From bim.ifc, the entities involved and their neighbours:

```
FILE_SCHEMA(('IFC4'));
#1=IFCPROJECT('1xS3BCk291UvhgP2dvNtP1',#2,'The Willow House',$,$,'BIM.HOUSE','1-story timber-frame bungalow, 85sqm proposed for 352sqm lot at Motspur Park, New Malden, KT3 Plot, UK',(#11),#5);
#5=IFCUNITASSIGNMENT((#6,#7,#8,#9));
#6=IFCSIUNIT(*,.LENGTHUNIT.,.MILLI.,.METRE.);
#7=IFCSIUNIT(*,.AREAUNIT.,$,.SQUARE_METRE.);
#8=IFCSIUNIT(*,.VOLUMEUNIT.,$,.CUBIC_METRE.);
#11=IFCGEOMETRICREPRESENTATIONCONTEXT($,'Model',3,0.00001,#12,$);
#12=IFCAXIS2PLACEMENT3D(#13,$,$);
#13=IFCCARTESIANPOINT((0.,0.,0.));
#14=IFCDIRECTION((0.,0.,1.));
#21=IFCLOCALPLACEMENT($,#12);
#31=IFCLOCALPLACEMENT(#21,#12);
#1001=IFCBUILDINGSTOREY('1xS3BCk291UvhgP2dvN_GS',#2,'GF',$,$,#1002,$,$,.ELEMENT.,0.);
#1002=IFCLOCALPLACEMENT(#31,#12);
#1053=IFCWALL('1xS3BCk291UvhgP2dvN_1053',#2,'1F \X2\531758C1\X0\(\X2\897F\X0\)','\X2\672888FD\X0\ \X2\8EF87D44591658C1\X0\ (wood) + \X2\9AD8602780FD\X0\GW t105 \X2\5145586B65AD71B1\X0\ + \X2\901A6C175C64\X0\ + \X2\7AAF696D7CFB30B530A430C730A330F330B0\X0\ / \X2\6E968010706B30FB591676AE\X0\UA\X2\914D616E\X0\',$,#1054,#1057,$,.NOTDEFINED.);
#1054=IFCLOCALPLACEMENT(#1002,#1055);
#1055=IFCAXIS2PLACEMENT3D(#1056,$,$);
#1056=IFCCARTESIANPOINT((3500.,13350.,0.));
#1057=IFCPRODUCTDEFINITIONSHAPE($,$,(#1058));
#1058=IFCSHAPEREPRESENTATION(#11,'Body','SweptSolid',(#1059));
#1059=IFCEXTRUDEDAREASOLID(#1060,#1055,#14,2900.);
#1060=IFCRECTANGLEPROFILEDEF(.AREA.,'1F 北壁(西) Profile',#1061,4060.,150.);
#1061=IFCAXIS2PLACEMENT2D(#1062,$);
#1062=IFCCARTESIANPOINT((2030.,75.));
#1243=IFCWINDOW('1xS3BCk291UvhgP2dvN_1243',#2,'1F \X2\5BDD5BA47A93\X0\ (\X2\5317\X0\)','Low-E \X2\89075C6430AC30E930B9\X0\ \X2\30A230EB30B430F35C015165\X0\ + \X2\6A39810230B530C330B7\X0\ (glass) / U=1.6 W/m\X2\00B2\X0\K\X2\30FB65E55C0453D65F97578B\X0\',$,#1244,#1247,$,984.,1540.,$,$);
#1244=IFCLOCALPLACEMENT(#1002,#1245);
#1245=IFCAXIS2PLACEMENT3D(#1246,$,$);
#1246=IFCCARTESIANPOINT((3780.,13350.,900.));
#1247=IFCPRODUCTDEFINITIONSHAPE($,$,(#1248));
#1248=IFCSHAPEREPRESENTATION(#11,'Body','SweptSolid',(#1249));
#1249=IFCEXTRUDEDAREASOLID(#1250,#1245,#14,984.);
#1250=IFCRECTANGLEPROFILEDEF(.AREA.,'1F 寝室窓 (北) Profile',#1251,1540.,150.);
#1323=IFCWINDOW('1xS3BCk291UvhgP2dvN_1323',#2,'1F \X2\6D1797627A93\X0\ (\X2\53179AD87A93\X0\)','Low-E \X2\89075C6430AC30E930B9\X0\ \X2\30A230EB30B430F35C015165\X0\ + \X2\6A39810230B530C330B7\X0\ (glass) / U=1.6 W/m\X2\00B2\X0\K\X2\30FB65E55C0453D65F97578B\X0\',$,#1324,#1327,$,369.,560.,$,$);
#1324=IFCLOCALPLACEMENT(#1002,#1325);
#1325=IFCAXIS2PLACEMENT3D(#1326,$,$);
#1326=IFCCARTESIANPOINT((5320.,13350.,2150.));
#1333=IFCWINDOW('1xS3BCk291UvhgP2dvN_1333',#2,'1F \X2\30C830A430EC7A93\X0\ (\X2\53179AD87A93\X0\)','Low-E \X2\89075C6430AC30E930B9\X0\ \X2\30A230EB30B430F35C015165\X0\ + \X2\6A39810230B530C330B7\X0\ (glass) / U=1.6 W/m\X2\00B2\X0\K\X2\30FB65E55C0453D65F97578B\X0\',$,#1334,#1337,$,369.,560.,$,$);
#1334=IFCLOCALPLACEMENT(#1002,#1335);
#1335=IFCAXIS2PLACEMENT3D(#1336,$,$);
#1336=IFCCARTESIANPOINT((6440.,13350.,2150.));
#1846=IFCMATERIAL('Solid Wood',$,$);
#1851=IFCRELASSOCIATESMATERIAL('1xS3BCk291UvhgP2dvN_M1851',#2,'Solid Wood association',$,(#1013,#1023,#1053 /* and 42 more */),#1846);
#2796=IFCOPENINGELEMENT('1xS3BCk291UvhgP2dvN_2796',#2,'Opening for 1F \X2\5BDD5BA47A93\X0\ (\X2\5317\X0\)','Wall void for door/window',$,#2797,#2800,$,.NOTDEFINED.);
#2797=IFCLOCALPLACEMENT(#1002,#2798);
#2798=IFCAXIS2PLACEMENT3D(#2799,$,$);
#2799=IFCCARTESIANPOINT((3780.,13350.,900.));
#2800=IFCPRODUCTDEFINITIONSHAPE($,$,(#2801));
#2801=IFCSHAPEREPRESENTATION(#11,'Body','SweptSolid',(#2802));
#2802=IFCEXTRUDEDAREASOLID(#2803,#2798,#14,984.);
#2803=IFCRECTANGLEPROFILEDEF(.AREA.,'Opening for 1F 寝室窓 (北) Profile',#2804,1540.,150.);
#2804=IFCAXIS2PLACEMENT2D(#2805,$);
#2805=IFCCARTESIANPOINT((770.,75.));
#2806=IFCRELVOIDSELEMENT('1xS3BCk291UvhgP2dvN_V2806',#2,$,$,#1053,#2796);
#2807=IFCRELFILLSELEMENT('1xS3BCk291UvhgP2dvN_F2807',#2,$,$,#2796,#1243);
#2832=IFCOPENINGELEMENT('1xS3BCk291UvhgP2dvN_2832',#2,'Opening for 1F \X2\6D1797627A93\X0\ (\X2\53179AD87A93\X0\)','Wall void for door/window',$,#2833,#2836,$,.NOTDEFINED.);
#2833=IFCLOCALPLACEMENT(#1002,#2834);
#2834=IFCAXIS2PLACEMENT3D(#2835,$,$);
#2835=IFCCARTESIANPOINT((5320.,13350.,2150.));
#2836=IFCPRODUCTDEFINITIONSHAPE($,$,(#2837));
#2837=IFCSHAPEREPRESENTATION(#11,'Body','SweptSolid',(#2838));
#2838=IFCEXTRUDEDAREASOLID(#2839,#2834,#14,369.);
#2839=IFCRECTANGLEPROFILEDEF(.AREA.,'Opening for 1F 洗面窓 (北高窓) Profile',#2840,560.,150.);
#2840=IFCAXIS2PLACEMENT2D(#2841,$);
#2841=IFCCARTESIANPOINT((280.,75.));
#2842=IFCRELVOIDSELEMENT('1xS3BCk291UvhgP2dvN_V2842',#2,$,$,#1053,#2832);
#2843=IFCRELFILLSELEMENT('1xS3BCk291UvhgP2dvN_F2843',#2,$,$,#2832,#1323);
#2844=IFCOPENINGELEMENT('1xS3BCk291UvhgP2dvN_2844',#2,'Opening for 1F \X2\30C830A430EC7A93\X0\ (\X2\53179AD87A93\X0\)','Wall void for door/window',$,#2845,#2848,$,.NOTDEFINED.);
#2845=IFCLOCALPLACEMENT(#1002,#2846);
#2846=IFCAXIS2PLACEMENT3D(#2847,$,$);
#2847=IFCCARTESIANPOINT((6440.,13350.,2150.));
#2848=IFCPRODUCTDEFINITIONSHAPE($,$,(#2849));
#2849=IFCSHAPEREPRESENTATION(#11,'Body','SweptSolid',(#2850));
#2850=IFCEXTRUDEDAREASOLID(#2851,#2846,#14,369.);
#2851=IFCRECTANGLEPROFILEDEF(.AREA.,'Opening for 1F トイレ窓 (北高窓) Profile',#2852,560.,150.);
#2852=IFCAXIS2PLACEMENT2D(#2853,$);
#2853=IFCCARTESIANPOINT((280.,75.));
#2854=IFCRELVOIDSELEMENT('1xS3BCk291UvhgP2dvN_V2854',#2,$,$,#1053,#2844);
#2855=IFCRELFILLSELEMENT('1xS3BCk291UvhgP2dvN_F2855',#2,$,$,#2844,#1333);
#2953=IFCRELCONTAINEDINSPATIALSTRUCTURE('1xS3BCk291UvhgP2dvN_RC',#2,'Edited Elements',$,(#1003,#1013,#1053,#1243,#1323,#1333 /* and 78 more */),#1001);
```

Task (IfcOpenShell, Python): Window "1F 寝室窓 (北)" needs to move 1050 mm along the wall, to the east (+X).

```python
import ifcopenshell
import ifcopenshell.api.geometry
import ifcopenshell.util.placement
import ifcopenshell.util.unit

model = ifcopenshell.open("bim.ifc")
unit_scale = ifcopenshell.util.unit.calculate_unit_scale(model)

window = model.by_guid("1xS3BCk291UvhgP2dvN_1243")
opening = window.FillsVoids[0].RelatingOpeningElement
wall = opening.VoidsElements[0].RelatingBuildingElement

wall_matrix = ifcopenshell.util.placement.get_local_placement(wall.ObjectPlacement)
shift = wall_matrix[:3, 0] * 1.05 / unit_scale
before = ifcopenshell.util.placement.get_local_placement(window.ObjectPlacement)[:3, 3].copy()

# The window is not placed relative to its opening, so move both.
for product in (opening, window):
    matrix = ifcopenshell.util.placement.get_local_placement(product.ObjectPlacement)
    matrix[:3, 3] += shift
    ifcopenshell.api.geometry.edit_object_placement(model, product=product, matrix=matrix, is_si=False)

after = ifcopenshell.util.placement.get_local_placement(window.ObjectPlacement)[:3, 3]
print("window moved by", (after - before).round(3) + 0.0)

model.write("bim_v2.ifc")
```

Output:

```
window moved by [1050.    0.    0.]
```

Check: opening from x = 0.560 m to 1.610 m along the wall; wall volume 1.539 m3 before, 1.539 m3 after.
